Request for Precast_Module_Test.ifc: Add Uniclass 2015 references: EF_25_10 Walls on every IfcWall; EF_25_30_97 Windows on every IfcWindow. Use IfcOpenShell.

First a look at what the model holds.

```python
import ifcopenshell

model = ifcopenshell.open("Precast_Module_Test.ifc")
print(model.schema)
print("classifications:", [c.Name for c in model.by_type("IfcClassification")])
for ifc_class in ("IfcDoor", "IfcRoof", "IfcStair", "IfcWall", "IfcWindow"):
    print(ifc_class, len(model.by_type(ifc_class)))
```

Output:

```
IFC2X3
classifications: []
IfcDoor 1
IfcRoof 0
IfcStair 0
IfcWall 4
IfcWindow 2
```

```python
import ifcopenshell
import ifcopenshell.api.classification

model = ifcopenshell.open("Precast_Module_Test.ifc")

# IFC2X3 requires Source and Edition and has no link from the project to the system.
system = model.create_entity("IfcClassification", Source="NBS", Edition="2015", Name="Uniclass 2015")

codes = {
    "IfcWall": ("EF_25_10", "Walls"),
    "IfcWindow": ("EF_25_30_97", "Windows"),
}
for ifc_class, (code, name) in codes.items():
    products = model.by_type(ifc_class)
    ifcopenshell.api.classification.add_reference(
        model, products=products, classification=system, identification=code, name=name
    )
    print(code, len(products))

model.write("Precast_Module_Test_rev.ifc")
```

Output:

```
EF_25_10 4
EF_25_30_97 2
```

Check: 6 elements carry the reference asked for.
